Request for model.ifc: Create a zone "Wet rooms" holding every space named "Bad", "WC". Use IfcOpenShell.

First a look at what the model holds.

```python
import ifcopenshell

model = ifcopenshell.open("model.ifc")
print(model.schema)
seen = {}
for space in model.by_type("IfcSpace"):
    seen[space.LongName] = seen.get(space.LongName, 0) + 1
for name, count in sorted(seen.items(), key=str):
    print(count, "x", name)
print("zones:", [z.Name for z in model.by_type("IfcZone")][:20])
```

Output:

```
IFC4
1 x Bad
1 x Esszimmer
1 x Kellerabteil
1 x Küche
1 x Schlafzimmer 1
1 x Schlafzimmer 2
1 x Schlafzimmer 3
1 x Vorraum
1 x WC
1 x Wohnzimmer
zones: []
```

```python
import ifcopenshell
import ifcopenshell.api.group
import ifcopenshell.api.root

model = ifcopenshell.open("model.ifc")

names = {"Bad", "WC"}
spaces = [s for s in model.by_type("IfcSpace") if s.LongName in names]

zone = ifcopenshell.api.root.create_entity(model, ifc_class="IfcZone", name="Wet rooms")
ifcopenshell.api.group.assign_group(model, products=spaces, group=zone)
print(len(spaces), "spaces in", zone.Name)

model.write("model_v2.ifc")
```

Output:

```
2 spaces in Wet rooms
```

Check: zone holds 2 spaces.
